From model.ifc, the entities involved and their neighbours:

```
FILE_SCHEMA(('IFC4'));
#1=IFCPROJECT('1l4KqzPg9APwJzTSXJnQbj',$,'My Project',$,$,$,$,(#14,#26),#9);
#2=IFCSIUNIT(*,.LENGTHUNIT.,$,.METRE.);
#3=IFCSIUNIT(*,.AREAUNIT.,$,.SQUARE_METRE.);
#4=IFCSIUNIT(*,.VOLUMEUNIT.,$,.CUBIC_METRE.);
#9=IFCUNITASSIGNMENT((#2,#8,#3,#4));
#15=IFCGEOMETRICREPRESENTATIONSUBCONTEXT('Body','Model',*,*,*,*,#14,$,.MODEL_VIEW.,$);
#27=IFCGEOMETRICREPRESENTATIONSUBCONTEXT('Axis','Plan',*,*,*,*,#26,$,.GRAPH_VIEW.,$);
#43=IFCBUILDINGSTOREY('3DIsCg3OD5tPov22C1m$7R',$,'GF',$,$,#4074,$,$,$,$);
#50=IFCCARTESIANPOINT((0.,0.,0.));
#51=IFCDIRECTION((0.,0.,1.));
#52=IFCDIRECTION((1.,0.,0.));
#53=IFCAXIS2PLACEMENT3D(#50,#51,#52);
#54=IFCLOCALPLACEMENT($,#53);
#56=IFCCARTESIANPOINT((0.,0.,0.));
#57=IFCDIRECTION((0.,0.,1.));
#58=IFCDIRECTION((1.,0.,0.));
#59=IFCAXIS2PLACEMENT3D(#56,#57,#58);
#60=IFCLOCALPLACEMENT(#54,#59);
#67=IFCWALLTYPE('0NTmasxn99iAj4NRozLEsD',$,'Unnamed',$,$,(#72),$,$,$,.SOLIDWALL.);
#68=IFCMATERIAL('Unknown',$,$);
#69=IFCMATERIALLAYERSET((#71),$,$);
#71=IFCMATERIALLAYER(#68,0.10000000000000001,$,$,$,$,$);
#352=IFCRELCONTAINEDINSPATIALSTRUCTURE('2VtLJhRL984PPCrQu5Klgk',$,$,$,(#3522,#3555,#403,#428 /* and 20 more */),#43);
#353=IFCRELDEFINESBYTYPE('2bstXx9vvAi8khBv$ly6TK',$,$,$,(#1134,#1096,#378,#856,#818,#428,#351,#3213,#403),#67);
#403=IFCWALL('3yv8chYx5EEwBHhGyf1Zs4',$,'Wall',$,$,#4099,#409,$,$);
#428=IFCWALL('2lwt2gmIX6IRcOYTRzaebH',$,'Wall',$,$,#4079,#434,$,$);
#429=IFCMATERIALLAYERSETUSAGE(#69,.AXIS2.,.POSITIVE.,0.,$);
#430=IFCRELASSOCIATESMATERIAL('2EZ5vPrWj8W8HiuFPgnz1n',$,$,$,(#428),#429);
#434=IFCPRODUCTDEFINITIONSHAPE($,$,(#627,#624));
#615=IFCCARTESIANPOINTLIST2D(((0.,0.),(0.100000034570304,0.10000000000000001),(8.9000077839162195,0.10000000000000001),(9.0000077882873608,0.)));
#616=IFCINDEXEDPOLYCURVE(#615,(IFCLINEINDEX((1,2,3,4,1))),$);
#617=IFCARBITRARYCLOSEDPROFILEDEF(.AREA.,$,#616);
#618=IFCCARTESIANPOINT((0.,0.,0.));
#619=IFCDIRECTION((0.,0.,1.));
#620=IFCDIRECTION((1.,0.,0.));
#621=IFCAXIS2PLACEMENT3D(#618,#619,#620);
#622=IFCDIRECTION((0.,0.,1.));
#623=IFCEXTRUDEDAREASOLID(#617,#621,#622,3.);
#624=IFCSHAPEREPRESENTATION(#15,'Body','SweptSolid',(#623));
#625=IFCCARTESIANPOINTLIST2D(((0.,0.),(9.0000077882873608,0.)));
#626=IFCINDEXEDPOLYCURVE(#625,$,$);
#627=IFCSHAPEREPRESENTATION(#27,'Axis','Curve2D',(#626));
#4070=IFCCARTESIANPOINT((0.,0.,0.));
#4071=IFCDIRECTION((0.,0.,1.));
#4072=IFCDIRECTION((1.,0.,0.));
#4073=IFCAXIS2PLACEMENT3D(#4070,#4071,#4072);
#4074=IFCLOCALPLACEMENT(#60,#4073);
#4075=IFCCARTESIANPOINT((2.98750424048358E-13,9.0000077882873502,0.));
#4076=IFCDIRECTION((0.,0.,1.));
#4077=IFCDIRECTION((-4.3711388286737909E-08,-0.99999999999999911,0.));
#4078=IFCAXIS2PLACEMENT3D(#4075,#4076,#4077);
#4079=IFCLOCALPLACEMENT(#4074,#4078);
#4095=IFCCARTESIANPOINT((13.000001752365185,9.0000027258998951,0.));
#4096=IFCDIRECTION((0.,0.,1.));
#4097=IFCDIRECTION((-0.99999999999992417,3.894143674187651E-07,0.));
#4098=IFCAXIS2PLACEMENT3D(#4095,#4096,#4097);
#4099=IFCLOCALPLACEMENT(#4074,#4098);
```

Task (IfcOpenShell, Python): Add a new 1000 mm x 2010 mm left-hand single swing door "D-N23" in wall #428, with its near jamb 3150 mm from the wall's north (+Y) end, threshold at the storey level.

```python
import numpy as np
import ifcopenshell
import ifcopenshell.api.feature
import ifcopenshell.api.geometry
import ifcopenshell.api.root
import ifcopenshell.api.spatial
import ifcopenshell.geom
import ifcopenshell.util.element
import ifcopenshell.util.placement
import ifcopenshell.util.representation
import ifcopenshell.util.shape
import ifcopenshell.util.unit

model = ifcopenshell.open("model.ifc")
unit_scale = ifcopenshell.util.unit.calculate_unit_scale(model)
settings = ifcopenshell.geom.settings()


def volume(element):
    """Net volume in cubic metres, openings subtracted."""
    shape = ifcopenshell.geom.create_shape(settings, element)
    return ifcopenshell.util.shape.get_volume(shape.geometry)


wall = model.by_id(428)
storey = ifcopenshell.util.element.get_container(wall, ifc_class="IfcBuildingStorey")
context = ifcopenshell.util.representation.get_context(model, "Model", "Body", "MODEL_VIEW")
before = volume(wall)

width, height, from_end, sill = 1, 2.01, 3.15, 0.0  # metres

# The wall runs along its own X axis, and the end named is its -X end.
wall_shape = ifcopenshell.geom.create_shape(settings, wall)
x, y, z = ifcopenshell.util.shape.get_vertices(wall_shape.geometry).T
start = x.min() + from_end
face, thickness = float(y.min()), float(y.max() - y.min())
wall_matrix = ifcopenshell.util.placement.get_local_placement(wall.ObjectPlacement)
level = ifcopenshell.util.placement.get_local_placement(storey.ObjectPlacement)[2, 3]


def in_wall(x, y):
    """Placement at x, y metres in the wall's axes, at sill height."""
    matrix = wall_matrix.copy()
    matrix[:, 3] = wall_matrix @ np.array([x / unit_scale, y / unit_scale, 0.0, 1.0])
    matrix[2, 3] = level + sill / unit_scale
    return matrix


# Opening: a box that overshoots both wall faces by 50 mm.
opening = ifcopenshell.api.root.create_entity(model, ifc_class="IfcOpeningElement", predefined_type="OPENING")
box = ifcopenshell.api.geometry.add_wall_representation(
    model, context=context, length=width, height=height, thickness=thickness + 0.1
)
ifcopenshell.api.geometry.assign_representation(model, product=opening, representation=box)
ifcopenshell.api.geometry.edit_object_placement(model, product=opening, matrix=in_wall(start, face - 0.05), is_si=False)
ifcopenshell.api.feature.add_feature(model, feature=opening, element=wall)

door = ifcopenshell.api.root.create_entity(model, ifc_class="IfcDoor", name="D-N23", predefined_type="DOOR")
door.OverallWidth, door.OverallHeight = width / unit_scale, height / unit_scale
door.OperationType = "SINGLE_SWING_LEFT"
body = ifcopenshell.api.geometry.add_door_representation(
    model,
    context=context,
    overall_width=door.OverallWidth,
    overall_height=door.OverallHeight,
    operation_type="SINGLE_SWING_LEFT",
    lining_properties={"LiningDepth": thickness / unit_scale, "ThresholdDepth": thickness / unit_scale},
)
ifcopenshell.api.geometry.assign_representation(model, product=door, representation=body)
ifcopenshell.api.spatial.assign_container(model, products=[door], relating_structure=storey)
ifcopenshell.api.feature.add_filling(model, opening=opening, element=door)

# The lining spans the wall, so the door starts at the wall face.
ifcopenshell.api.geometry.edit_object_placement(model, product=door, matrix=in_wall(start, face), is_si=False)

after = volume(wall)

print(f"wall volume {before:.3f} -> {after:.3f} m3")

model.write("model_updated.ifc")
```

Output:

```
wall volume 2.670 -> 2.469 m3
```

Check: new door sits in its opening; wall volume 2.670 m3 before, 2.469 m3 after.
